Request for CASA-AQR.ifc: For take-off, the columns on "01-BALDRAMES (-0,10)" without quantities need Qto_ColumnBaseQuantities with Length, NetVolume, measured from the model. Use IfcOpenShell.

First a look at what the model holds.

```python
import ifcopenshell
import ifcopenshell.util.element
import ifcopenshell.util.unit

model = ifcopenshell.open("CASA-AQR.ifc")
print(model.schema)
for unit_type in ("LENGTHUNIT", "AREAUNIT", "VOLUMEUNIT"):
    print(unit_type, ifcopenshell.util.unit.calculate_unit_scale(model, unit_type))
storey = next(s for s in model.by_type("IfcBuildingStorey") if s.Name == "01-BALDRAMES (-0,10)")
columns = [e for e in ifcopenshell.util.element.get_decomposition(storey) if e.is_a("IfcColumn")]
for e in sorted(columns, key=lambda e: e.id()):
    print(e.id(), e.is_a(), e.Name, list(ifcopenshell.util.element.get_psets(e, qtos_only=True)), sep=" | ")
```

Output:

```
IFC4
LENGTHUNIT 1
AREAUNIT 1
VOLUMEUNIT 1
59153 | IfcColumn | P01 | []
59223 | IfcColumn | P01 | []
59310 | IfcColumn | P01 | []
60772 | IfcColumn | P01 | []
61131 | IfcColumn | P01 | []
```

```python
import ifcopenshell
import ifcopenshell.api.pset
import ifcopenshell.geom
import ifcopenshell.util.element
import ifcopenshell.util.shape
import ifcopenshell.util.unit

model = ifcopenshell.open("CASA-AQR.ifc")
unit_scale = ifcopenshell.util.unit.calculate_unit_scale(model)
volume_scale = ifcopenshell.util.unit.calculate_unit_scale(model, "VOLUMEUNIT")
settings = ifcopenshell.geom.settings()

storey = next(s for s in model.by_type("IfcBuildingStorey") if s.Name == "01-BALDRAMES (-0,10)")
columns = [e for e in ifcopenshell.util.element.get_decomposition(storey) if e.is_a("IfcColumn")]

for e in sorted(columns, key=lambda e: e.id()):
    if ifcopenshell.util.element.get_psets(e, qtos_only=True, should_inherit=False):
        continue
    # Geometry comes back in metres, in the element's own axes.
    shape = ifcopenshell.geom.create_shape(settings, e)
    values = {
        "Length": ifcopenshell.util.shape.get_z(shape.geometry) / unit_scale,
        "NetVolume": ifcopenshell.util.shape.get_volume(shape.geometry) / volume_scale,
    }
    qto = ifcopenshell.api.pset.add_qto(model, product=e, name="Qto_ColumnBaseQuantities")
    ifcopenshell.api.pset.edit_qto(model, qto=qto, properties=values)
    print(e.id(), {k: round(v, 3) for k, v in values.items()})

model.write("CASA-AQR_edited.ifc")
```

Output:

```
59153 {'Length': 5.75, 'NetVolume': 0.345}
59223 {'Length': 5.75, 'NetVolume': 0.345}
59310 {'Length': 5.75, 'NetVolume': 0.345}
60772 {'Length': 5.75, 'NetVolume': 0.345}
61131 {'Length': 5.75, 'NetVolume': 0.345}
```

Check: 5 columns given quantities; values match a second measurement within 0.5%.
